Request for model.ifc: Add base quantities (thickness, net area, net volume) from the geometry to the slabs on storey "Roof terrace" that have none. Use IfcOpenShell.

First a look at what the model holds.

```python
import ifcopenshell
import ifcopenshell.util.element
import ifcopenshell.util.unit

model = ifcopenshell.open("model.ifc")
print(model.schema)
for unit_type in ("LENGTHUNIT", "AREAUNIT", "VOLUMEUNIT"):
    print(unit_type, ifcopenshell.util.unit.calculate_unit_scale(model, unit_type))
storey = next(s for s in model.by_type("IfcBuildingStorey") if s.Name == "Roof terrace")
slabs = [e for e in ifcopenshell.util.element.get_decomposition(storey) if e.is_a("IfcSlab")]
for e in sorted(slabs, key=lambda e: e.id()):
    print(e.id(), e.is_a(), e.Name, list(ifcopenshell.util.element.get_psets(e, qtos_only=True)), sep=" | ")
```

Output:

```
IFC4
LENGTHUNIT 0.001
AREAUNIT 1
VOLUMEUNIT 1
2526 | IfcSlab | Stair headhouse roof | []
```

```python
import ifcopenshell
import ifcopenshell.api.pset
import ifcopenshell.geom
import ifcopenshell.util.element
import ifcopenshell.util.shape
import ifcopenshell.util.unit

model = ifcopenshell.open("model.ifc")
unit_scale = ifcopenshell.util.unit.calculate_unit_scale(model)
area_scale = ifcopenshell.util.unit.calculate_unit_scale(model, "AREAUNIT")
volume_scale = ifcopenshell.util.unit.calculate_unit_scale(model, "VOLUMEUNIT")
settings = ifcopenshell.geom.settings()

storey = next(s for s in model.by_type("IfcBuildingStorey") if s.Name == "Roof terrace")
slabs = [e for e in ifcopenshell.util.element.get_decomposition(storey) if e.is_a("IfcSlab")]

for e in sorted(slabs, key=lambda e: e.id()):
    if ifcopenshell.util.element.get_psets(e, qtos_only=True, should_inherit=False):
        continue
    # Geometry comes back in metres, in the element's own axes.
    shape = ifcopenshell.geom.create_shape(settings, e)
    values = {
        "Width": ifcopenshell.util.shape.get_z(shape.geometry) / unit_scale,
        "NetArea": ifcopenshell.util.shape.get_footprint_area(shape.geometry) / area_scale,
        "NetVolume": ifcopenshell.util.shape.get_volume(shape.geometry) / volume_scale,
    }
    qto = ifcopenshell.api.pset.add_qto(model, product=e, name="Qto_SlabBaseQuantities")
    ifcopenshell.api.pset.edit_qto(model, qto=qto, properties=values)
    print(e.id(), {k: round(v, 3) for k, v in values.items()})

model.write("model_rev.ifc")
```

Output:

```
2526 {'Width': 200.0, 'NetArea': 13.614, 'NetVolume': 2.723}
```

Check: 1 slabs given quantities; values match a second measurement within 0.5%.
